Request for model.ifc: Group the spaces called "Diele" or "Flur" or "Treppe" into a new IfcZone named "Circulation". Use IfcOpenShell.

First a look at what the model holds.

```python
import ifcopenshell

model = ifcopenshell.open("model.ifc")
print(model.schema)
seen = {}
for space in model.by_type("IfcSpace"):
    seen[space.LongName] = seen.get(space.LongName, 0) + 1
for name, count in sorted(seen.items(), key=str):
    print(count, "x", name)
print("zones:", [z.Name for z in model.by_type("IfcZone")][:20])
```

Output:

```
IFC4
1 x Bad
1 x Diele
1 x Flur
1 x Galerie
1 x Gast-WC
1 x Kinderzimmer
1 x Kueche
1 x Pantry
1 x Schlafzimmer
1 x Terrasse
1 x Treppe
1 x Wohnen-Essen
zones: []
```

```python
import ifcopenshell
import ifcopenshell.api.group
import ifcopenshell.api.root

model = ifcopenshell.open("model.ifc")

names = {"Diele", "Flur", "Treppe"}
spaces = [s for s in model.by_type("IfcSpace") if s.LongName in names]

zone = ifcopenshell.api.root.create_entity(model, ifc_class="IfcZone", name="Circulation")
ifcopenshell.api.group.assign_group(model, products=spaces, group=zone)
print(len(spaces), "spaces in", zone.Name)

model.write("model_v2.ifc")
```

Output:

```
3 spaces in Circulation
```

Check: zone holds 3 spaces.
